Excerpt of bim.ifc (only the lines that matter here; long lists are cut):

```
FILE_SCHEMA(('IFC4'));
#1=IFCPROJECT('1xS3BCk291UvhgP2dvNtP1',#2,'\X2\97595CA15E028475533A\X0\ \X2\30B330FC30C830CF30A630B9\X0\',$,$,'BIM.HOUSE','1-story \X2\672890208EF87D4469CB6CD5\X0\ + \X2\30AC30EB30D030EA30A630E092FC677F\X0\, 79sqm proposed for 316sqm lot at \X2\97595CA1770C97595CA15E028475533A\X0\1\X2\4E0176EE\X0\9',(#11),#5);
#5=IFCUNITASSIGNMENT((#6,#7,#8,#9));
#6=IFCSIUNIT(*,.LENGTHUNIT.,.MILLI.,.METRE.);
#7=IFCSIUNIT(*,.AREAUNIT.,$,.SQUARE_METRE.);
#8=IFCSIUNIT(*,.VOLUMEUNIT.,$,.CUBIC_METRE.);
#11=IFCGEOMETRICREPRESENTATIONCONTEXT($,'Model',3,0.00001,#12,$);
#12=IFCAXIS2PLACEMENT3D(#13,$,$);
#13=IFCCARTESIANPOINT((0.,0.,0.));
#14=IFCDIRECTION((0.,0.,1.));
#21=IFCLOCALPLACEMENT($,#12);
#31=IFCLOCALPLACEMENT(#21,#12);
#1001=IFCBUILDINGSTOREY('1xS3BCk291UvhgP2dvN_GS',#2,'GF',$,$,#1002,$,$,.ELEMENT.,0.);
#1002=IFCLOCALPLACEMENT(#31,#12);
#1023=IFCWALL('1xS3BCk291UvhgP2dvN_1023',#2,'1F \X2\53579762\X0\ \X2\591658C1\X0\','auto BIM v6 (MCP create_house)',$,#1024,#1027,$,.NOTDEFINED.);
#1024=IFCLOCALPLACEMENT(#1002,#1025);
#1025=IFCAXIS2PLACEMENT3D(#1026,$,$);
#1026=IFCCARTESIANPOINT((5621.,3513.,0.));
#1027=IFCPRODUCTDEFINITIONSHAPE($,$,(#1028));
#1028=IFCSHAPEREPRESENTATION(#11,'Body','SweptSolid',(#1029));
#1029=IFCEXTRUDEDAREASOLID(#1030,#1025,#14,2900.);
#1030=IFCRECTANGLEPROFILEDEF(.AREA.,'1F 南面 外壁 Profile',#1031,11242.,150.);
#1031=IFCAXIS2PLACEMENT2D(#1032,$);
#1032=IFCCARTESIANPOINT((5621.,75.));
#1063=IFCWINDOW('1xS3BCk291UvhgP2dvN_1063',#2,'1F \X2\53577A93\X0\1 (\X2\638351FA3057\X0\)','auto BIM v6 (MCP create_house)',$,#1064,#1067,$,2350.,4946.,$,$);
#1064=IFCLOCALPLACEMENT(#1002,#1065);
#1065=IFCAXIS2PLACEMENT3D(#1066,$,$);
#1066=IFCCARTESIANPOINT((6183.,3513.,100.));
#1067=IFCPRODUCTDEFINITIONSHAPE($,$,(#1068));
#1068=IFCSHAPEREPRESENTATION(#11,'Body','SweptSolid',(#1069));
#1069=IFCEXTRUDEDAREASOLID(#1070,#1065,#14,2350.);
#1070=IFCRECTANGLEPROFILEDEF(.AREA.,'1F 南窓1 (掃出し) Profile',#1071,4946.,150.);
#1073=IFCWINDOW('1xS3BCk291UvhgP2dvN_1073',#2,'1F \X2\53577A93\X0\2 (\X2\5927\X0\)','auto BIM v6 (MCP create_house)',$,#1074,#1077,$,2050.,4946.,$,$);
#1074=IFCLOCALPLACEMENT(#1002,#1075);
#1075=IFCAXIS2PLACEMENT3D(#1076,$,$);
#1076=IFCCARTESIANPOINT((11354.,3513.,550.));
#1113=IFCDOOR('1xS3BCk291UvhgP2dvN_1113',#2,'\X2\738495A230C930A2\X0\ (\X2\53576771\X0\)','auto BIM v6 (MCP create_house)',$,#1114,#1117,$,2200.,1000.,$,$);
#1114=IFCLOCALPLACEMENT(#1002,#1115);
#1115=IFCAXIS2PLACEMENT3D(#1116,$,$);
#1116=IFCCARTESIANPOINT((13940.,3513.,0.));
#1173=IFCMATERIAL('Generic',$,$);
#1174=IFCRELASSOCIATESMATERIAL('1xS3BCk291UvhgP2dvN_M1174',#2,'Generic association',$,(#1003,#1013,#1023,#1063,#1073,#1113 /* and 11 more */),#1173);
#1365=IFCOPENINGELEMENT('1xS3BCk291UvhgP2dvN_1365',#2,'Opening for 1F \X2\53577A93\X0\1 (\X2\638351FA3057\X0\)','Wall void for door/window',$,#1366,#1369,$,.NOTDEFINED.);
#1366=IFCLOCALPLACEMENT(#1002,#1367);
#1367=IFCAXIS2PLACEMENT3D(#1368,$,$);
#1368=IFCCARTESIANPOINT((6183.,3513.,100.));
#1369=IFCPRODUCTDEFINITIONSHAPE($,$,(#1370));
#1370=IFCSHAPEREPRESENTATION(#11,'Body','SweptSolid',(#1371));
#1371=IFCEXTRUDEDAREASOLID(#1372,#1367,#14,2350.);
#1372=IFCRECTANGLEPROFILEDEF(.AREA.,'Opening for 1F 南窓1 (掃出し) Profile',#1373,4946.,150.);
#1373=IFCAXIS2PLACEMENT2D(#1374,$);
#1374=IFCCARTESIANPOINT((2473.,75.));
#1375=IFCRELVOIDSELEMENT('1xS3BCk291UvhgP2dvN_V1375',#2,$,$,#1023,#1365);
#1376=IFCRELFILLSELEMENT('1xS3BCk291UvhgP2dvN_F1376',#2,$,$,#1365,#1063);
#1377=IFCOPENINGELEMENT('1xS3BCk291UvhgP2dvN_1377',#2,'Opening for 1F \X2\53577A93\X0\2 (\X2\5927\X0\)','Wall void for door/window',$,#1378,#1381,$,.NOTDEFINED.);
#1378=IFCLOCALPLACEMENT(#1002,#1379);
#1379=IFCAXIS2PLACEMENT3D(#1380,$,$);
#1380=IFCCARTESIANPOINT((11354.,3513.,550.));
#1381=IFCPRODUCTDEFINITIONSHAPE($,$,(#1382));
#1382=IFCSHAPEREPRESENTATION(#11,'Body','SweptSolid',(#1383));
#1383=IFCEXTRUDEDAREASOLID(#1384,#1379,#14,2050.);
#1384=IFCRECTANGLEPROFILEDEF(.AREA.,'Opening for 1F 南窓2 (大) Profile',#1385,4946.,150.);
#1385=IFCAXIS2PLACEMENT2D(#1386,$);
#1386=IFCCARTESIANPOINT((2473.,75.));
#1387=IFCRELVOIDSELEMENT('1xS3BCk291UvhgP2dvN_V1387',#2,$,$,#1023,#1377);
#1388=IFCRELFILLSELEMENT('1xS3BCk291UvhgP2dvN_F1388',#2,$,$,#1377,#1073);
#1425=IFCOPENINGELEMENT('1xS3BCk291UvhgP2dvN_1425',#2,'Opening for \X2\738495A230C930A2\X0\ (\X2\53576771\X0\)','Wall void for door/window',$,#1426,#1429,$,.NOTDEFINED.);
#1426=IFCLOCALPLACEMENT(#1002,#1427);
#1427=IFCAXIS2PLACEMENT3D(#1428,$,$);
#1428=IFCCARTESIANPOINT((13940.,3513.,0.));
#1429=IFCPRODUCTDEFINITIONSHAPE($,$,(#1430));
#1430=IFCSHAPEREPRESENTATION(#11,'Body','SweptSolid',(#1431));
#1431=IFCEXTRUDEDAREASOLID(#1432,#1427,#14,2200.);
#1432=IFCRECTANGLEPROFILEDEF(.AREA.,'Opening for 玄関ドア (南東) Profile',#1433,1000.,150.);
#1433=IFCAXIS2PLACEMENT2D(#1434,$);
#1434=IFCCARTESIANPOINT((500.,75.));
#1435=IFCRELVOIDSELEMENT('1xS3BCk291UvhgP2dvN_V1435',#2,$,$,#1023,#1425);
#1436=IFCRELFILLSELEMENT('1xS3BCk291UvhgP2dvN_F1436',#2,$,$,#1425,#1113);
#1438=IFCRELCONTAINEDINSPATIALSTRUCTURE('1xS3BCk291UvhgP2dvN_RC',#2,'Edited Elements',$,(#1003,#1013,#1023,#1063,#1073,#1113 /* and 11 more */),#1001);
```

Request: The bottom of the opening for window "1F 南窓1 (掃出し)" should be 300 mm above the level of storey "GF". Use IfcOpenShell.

```python
import numpy as np
import ifcopenshell
import ifcopenshell.api.geometry
import ifcopenshell.geom
import ifcopenshell.util.element
import ifcopenshell.util.placement
import ifcopenshell.util.shape
import ifcopenshell.util.unit

model = ifcopenshell.open("bim.ifc")
unit_scale = ifcopenshell.util.unit.calculate_unit_scale(model)

window = model.by_guid("1xS3BCk291UvhgP2dvN_1063")
opening = window.FillsVoids[0].RelatingOpeningElement
storey = ifcopenshell.util.element.get_container(window, ifc_class="IfcBuildingStorey")
level = ifcopenshell.util.placement.get_local_placement(storey.ObjectPlacement)[2, 3]

# The opening's origin need not be at the sill, so measure its lowest point.
shape = ifcopenshell.geom.create_shape(ifcopenshell.geom.settings(), opening)
bottom = ifcopenshell.util.shape.get_shape_bottom_elevation(shape, shape.geometry) / unit_scale
dz = level + 0.3 / unit_scale - bottom

shift = np.array([0.0, 0.0, dz])
# The window is not placed relative to its opening, so move both.
for product in (opening, window):
    matrix = ifcopenshell.util.placement.get_local_placement(product.ObjectPlacement)
    matrix[:3, 3] += shift
    ifcopenshell.api.geometry.edit_object_placement(model, product=product, matrix=matrix, is_si=False)

print(f"moved by {dz * unit_scale:+.3f} m")

model.write("bim_edited.ifc")
```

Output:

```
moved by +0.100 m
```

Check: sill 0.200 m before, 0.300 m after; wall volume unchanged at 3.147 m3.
